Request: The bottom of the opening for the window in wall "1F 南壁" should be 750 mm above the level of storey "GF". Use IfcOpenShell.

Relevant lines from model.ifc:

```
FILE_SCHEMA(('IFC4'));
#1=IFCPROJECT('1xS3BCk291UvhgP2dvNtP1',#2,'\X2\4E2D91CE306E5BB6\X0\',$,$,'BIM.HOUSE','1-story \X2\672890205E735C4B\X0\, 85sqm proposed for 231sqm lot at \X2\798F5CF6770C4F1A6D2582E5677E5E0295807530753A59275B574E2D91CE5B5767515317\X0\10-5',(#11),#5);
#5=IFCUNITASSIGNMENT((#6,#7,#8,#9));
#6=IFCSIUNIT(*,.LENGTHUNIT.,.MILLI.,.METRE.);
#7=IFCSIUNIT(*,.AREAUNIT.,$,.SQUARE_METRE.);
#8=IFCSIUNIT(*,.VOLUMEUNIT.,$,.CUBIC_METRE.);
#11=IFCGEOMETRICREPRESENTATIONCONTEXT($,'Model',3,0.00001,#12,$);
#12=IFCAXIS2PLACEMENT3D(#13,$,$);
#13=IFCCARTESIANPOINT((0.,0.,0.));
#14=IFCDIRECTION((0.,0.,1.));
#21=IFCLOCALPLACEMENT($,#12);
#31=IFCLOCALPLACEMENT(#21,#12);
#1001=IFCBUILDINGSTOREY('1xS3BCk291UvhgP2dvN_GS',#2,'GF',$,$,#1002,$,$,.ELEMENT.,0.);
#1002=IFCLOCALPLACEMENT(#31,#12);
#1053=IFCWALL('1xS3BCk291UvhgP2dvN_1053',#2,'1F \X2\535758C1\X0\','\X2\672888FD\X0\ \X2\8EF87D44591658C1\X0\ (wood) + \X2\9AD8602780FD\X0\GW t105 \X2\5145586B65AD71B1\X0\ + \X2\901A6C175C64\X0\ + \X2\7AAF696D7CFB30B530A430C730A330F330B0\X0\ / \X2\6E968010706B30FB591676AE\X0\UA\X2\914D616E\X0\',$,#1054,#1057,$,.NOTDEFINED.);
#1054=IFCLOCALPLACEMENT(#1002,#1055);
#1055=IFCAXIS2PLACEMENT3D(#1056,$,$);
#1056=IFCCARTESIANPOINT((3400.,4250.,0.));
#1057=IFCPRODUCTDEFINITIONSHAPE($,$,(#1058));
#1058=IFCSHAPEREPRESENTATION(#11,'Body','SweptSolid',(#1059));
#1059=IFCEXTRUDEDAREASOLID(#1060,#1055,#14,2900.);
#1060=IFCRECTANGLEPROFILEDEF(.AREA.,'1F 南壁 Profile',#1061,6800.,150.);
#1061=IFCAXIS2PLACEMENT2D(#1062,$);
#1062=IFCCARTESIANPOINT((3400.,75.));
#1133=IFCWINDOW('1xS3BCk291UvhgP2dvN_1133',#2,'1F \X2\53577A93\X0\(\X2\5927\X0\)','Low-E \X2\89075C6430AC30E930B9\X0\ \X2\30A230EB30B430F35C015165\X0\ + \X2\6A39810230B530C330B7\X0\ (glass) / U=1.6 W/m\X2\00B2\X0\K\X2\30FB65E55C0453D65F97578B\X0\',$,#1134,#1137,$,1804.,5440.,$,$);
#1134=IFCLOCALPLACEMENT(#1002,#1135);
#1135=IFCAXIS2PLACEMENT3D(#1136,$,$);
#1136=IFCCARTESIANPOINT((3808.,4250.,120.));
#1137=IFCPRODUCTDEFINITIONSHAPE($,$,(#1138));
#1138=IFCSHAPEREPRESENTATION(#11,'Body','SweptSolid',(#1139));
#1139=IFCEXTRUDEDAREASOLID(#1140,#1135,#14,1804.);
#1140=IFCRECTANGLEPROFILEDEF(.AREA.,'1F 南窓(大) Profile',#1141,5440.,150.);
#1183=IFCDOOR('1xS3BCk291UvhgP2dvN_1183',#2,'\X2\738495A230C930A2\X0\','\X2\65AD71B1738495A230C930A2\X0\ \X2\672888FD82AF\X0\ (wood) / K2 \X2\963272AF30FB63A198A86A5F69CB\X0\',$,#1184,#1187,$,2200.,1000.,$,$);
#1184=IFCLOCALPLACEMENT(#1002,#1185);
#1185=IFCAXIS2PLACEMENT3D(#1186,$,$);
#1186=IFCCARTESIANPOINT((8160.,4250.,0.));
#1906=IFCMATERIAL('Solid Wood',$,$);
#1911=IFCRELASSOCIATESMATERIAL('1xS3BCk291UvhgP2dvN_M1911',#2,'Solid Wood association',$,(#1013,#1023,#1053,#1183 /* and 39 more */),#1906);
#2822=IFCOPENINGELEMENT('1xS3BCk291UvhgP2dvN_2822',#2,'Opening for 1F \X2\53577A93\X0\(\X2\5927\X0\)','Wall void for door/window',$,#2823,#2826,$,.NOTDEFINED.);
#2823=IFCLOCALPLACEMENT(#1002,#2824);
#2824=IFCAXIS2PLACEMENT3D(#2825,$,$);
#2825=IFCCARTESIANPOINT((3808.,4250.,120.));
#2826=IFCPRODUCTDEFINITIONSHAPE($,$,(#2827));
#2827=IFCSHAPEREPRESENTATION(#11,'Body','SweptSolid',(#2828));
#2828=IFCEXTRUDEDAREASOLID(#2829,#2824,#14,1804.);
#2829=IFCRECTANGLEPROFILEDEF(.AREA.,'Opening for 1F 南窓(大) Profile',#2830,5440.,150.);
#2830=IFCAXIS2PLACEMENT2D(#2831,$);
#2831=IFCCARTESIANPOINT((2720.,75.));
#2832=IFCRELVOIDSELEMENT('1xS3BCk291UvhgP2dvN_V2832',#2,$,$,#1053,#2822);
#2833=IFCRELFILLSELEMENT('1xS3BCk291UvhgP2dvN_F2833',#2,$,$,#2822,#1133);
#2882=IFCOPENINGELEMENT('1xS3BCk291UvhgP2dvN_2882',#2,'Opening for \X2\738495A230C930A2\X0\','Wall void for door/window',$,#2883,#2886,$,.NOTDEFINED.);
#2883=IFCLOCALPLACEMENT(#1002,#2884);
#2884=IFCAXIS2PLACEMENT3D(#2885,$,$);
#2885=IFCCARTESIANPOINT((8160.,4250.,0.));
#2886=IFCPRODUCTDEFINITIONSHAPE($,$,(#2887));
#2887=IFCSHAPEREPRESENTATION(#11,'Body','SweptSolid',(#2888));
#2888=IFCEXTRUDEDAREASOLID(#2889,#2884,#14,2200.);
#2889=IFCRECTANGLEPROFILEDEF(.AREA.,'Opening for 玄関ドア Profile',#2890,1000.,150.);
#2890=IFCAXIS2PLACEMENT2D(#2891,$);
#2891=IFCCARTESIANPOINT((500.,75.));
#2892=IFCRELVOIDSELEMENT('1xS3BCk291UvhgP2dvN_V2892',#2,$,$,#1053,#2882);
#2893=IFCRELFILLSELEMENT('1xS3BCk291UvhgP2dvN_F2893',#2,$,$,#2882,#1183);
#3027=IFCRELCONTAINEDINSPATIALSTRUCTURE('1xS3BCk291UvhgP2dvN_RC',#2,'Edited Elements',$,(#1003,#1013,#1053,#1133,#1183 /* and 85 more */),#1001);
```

```python
import numpy as np
import ifcopenshell
import ifcopenshell.api.geometry
import ifcopenshell.geom
import ifcopenshell.util.element
import ifcopenshell.util.placement
import ifcopenshell.util.shape
import ifcopenshell.util.unit

model = ifcopenshell.open("model.ifc")
unit_scale = ifcopenshell.util.unit.calculate_unit_scale(model)

window = model.by_guid("1xS3BCk291UvhgP2dvN_1133")
opening = window.FillsVoids[0].RelatingOpeningElement
storey = ifcopenshell.util.element.get_container(window, ifc_class="IfcBuildingStorey")
level = ifcopenshell.util.placement.get_local_placement(storey.ObjectPlacement)[2, 3]

# The opening's origin need not be at the sill, so measure its lowest point.
shape = ifcopenshell.geom.create_shape(ifcopenshell.geom.settings(), opening)
bottom = ifcopenshell.util.shape.get_shape_bottom_elevation(shape, shape.geometry) / unit_scale
dz = level + 750.0 - bottom

shift = np.array([0.0, 0.0, dz])
# The window is not placed relative to its opening, so move both.
for product in (opening, window):
    matrix = ifcopenshell.util.placement.get_local_placement(product.ObjectPlacement)
    matrix[:3, 3] += shift
    ifcopenshell.api.geometry.edit_object_placement(model, product=product, matrix=matrix, is_si=False)

print(f"moved by {dz * unit_scale:+.3f} m")

model.write("model_rev.ifc")
```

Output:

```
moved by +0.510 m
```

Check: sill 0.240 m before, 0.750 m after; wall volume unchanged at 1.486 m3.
